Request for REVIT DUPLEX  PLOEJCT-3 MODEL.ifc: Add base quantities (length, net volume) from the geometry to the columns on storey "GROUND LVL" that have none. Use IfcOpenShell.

First a look at what the model holds.

```python
import ifcopenshell
import ifcopenshell.util.element
import ifcopenshell.util.unit

model = ifcopenshell.open("REVIT DUPLEX  PLOEJCT-3 MODEL.ifc")
print(model.schema)
for unit_type in ("LENGTHUNIT", "AREAUNIT", "VOLUMEUNIT"):
    print(unit_type, ifcopenshell.util.unit.calculate_unit_scale(model, unit_type))
storey = next(s for s in model.by_type("IfcBuildingStorey") if s.Name == "GROUND LVL")
columns = [e for e in ifcopenshell.util.element.get_decomposition(storey) if e.is_a("IfcColumn")]
for e in sorted(columns, key=lambda e: e.id()):
    print(e.id(), e.is_a(), e.Name, list(ifcopenshell.util.element.get_psets(e, qtos_only=True)), sep=" | ")
```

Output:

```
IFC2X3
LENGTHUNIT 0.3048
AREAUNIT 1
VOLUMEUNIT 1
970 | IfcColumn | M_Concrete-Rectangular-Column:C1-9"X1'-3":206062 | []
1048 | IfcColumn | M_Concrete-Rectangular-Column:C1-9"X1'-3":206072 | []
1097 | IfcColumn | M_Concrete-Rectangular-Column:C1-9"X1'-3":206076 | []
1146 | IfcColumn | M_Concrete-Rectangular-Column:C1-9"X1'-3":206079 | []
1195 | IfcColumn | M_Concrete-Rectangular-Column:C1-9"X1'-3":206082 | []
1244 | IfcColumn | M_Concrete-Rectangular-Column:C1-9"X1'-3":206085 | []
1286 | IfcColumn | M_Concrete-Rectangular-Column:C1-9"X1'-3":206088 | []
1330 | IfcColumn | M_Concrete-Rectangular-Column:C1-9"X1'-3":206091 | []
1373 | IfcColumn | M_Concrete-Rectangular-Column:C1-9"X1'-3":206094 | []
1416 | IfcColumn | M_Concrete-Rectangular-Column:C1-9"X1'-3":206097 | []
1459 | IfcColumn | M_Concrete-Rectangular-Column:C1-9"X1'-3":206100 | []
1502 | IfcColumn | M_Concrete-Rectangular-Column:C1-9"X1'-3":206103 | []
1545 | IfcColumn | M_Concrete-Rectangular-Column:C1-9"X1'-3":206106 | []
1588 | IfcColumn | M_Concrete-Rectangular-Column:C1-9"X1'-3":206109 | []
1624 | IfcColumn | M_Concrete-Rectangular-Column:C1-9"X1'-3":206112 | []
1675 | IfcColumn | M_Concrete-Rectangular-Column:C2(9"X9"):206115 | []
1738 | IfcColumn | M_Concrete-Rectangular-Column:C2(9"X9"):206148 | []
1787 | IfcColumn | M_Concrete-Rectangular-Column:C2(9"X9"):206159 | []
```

```python
import ifcopenshell
import ifcopenshell.api.pset
import ifcopenshell.geom
import ifcopenshell.util.element
import ifcopenshell.util.shape
import ifcopenshell.util.unit

model = ifcopenshell.open("REVIT DUPLEX  PLOEJCT-3 MODEL.ifc")
unit_scale = ifcopenshell.util.unit.calculate_unit_scale(model)
volume_scale = ifcopenshell.util.unit.calculate_unit_scale(model, "VOLUMEUNIT")
settings = ifcopenshell.geom.settings()

storey = next(s for s in model.by_type("IfcBuildingStorey") if s.Name == "GROUND LVL")
columns = [e for e in ifcopenshell.util.element.get_decomposition(storey) if e.is_a("IfcColumn")]

for e in sorted(columns, key=lambda e: e.id()):
    if ifcopenshell.util.element.get_psets(e, qtos_only=True, should_inherit=False):
        continue
    # Geometry comes back in metres, in the element's own axes.
    shape = ifcopenshell.geom.create_shape(settings, e)
    values = {
        "Length": ifcopenshell.util.shape.get_z(shape.geometry) / unit_scale,
        "NetVolume": ifcopenshell.util.shape.get_volume(shape.geometry) / volume_scale,
    }
    qto = ifcopenshell.api.pset.add_qto(model, product=e, name="BaseQuantities")
    ifcopenshell.api.pset.edit_qto(model, qto=qto, properties=values)
    print(e.id(), {k: round(v, 3) for k, v in values.items()})

model.write("REVIT DUPLEX  PLOEJCT-3 MODEL_edited.ifc")
```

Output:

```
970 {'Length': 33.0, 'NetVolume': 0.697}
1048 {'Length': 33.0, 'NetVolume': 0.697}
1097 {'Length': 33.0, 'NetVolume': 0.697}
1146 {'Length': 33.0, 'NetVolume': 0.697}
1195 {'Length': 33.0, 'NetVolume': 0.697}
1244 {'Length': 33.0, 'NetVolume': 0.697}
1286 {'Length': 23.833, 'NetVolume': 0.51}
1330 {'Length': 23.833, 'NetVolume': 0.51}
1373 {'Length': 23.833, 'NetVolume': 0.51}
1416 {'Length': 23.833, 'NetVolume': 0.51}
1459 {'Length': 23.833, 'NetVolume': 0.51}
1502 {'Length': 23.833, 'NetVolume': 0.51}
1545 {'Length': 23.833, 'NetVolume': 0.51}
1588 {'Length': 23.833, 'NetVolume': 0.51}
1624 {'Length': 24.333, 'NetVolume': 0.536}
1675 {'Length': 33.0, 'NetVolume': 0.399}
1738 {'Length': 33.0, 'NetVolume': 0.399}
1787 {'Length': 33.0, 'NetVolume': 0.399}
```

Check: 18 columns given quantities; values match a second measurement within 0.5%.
